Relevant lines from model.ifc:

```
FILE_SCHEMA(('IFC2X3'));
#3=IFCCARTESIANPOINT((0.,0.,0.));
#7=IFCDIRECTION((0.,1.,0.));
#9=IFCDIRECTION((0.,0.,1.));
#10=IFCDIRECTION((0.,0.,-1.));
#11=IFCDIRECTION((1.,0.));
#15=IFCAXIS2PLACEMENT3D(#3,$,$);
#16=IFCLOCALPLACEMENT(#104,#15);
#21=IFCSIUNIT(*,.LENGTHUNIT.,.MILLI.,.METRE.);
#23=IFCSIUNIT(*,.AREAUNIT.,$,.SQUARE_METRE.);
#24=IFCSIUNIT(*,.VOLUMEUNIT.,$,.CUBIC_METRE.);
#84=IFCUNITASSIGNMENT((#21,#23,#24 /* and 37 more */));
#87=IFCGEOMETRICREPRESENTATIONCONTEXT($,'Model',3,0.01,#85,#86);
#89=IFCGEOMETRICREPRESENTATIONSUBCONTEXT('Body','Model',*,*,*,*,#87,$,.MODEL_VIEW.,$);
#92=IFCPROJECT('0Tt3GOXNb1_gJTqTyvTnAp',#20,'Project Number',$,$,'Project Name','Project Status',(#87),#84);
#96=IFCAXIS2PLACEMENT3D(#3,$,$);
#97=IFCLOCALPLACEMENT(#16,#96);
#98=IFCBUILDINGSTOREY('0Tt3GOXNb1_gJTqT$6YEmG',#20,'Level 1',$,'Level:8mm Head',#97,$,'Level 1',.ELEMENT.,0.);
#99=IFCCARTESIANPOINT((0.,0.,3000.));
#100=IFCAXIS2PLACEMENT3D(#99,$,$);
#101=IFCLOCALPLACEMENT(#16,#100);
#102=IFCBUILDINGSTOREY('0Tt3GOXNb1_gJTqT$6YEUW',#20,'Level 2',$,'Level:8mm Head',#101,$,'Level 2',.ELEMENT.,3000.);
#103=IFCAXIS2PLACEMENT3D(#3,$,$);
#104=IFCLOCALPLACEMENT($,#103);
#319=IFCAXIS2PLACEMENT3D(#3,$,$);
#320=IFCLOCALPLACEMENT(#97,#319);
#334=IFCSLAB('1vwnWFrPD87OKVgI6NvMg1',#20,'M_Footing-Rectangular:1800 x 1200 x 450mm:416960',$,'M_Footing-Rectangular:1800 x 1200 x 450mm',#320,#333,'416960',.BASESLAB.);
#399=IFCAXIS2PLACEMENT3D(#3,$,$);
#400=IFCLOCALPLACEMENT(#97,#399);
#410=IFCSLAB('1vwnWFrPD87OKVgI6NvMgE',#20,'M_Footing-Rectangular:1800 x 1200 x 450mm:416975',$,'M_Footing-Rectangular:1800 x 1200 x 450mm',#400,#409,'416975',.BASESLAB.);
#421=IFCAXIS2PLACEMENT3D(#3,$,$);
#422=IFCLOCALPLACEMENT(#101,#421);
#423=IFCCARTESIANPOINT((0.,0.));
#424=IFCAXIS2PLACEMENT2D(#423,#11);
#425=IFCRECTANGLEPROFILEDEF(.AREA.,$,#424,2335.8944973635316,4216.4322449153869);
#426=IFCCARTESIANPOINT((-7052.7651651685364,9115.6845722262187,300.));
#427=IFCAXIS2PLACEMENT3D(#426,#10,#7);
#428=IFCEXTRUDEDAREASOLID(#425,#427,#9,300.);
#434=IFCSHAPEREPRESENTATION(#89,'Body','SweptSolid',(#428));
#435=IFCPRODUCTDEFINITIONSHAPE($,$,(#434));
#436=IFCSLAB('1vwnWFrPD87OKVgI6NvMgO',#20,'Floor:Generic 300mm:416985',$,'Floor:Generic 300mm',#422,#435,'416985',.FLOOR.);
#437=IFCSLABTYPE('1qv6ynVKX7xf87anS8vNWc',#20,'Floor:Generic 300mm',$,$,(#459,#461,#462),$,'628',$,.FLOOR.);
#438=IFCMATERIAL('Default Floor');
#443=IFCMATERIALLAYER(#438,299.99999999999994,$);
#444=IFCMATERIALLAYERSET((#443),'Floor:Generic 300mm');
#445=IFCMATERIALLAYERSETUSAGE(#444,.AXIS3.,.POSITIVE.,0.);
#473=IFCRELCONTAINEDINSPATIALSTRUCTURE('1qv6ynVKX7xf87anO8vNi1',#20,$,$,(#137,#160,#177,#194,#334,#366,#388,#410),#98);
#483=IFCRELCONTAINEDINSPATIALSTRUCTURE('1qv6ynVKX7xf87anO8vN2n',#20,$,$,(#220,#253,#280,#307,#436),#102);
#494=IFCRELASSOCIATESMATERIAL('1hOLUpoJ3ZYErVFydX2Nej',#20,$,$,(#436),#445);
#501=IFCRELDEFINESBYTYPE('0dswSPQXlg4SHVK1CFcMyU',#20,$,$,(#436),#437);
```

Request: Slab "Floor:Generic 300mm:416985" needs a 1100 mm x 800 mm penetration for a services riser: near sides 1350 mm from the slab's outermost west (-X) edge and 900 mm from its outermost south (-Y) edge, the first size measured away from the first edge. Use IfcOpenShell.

```python
import numpy as np
import ifcopenshell
import ifcopenshell.api.feature
import ifcopenshell.api.geometry
import ifcopenshell.api.root
import ifcopenshell.geom
import ifcopenshell.util.placement
import ifcopenshell.util.representation
import ifcopenshell.util.shape
import ifcopenshell.util.unit

model = ifcopenshell.open("model.ifc")
unit_scale = ifcopenshell.util.unit.calculate_unit_scale(model)
settings = ifcopenshell.geom.settings()


def volume(element):
    """Net volume in cubic metres, openings subtracted."""
    shape = ifcopenshell.geom.create_shape(settings, element)
    return ifcopenshell.util.shape.get_volume(shape.geometry)


slab = model.by_id(436)
before = volume(slab)

# Extent in the slab's own axes, in metres. The edges named are its -X and -Y sides.
slab_shape = ifcopenshell.geom.create_shape(settings, slab)
vertices = ifcopenshell.util.shape.get_vertices(slab_shape.geometry)
x_min, y_min, bottom = vertices.min(axis=0)
top = vertices[:, 2].max()

opening = ifcopenshell.api.root.create_entity(model, ifc_class="IfcOpeningElement", name="Services riser opening")
context = ifcopenshell.util.representation.get_context(model, "Model", "Body", "MODEL_VIEW")
width, depth = 1.1, 0.8
outline = [(0.0, 0.0), (width, 0.0), (width, depth), (0.0, depth), (0.0, 0.0)]
# Overshoot both faces by 50 mm so the cut is clean.
shape = ifcopenshell.api.geometry.add_slab_representation(
    model, context=context, depth=top - bottom + 0.1, polyline=outline
)
ifcopenshell.api.geometry.assign_representation(model, product=opening, representation=shape)

matrix = ifcopenshell.util.placement.get_local_placement(slab.ObjectPlacement)
matrix[:, 3] = matrix @ np.append(np.array([x_min + 1.35, y_min + 0.9, bottom - 0.05]) / unit_scale, 1.0)
ifcopenshell.api.geometry.edit_object_placement(model, product=opening, matrix=matrix, is_si=False)
ifcopenshell.api.feature.add_feature(model, feature=opening, element=slab)

after = volume(slab)

print(f"slab volume {before:.3f} -> {after:.3f} m3")

model.write("model_rev.ifc")
```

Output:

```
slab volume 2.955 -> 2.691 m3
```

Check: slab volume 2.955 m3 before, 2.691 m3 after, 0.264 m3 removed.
